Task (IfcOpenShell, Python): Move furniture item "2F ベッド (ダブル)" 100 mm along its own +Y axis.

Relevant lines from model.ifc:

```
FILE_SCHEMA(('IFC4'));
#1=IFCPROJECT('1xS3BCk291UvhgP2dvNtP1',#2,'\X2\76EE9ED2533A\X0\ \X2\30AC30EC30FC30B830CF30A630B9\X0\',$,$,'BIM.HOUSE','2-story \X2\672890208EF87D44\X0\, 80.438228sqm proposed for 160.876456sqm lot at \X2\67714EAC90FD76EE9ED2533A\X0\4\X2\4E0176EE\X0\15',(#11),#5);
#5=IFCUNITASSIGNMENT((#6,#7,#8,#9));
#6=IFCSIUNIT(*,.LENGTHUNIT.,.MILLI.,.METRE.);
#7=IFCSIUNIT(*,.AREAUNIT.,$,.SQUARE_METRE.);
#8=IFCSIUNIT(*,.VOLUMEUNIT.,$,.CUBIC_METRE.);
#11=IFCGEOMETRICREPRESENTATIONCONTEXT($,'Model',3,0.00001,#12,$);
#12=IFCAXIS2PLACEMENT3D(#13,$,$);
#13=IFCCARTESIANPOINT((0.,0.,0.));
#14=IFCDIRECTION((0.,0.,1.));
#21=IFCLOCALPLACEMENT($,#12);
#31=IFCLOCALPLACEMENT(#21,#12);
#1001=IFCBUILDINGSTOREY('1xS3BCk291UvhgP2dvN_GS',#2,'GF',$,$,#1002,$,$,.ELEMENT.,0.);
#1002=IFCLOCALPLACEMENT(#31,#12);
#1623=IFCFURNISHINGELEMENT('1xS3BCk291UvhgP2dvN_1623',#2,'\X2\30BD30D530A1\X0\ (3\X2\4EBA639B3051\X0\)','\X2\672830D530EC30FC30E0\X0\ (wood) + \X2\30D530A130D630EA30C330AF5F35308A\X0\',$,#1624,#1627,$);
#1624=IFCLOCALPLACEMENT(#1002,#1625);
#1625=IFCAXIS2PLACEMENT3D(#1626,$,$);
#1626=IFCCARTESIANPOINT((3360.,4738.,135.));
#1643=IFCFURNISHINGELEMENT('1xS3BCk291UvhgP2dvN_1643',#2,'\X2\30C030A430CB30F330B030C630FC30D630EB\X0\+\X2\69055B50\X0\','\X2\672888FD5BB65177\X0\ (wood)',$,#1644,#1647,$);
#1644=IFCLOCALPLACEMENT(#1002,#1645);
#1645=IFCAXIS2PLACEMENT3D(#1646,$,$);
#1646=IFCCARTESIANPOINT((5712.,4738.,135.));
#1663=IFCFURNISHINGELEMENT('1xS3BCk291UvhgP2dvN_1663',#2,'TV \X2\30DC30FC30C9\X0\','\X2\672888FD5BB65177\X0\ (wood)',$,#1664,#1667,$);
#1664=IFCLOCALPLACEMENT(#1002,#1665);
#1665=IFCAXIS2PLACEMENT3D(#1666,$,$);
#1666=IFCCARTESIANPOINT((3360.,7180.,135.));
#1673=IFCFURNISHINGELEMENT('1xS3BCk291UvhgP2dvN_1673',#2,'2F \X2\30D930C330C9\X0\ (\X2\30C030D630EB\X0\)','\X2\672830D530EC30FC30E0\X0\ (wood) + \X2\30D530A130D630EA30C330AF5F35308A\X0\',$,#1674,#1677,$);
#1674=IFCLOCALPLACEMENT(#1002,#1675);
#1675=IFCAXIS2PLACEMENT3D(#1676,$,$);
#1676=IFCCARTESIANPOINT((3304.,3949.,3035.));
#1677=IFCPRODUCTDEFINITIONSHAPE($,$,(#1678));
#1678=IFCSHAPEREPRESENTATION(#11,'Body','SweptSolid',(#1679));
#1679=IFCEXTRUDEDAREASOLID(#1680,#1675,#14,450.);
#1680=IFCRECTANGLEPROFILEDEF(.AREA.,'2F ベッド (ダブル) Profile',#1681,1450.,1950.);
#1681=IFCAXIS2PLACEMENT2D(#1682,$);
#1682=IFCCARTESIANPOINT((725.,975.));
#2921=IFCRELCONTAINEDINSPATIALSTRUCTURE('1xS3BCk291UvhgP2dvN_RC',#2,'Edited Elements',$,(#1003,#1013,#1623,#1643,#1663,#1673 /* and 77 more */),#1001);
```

```python
import ifcopenshell
import ifcopenshell.api.geometry
import ifcopenshell.util.placement
import ifcopenshell.util.unit

model = ifcopenshell.open("model.ifc")
unit_scale = ifcopenshell.util.unit.calculate_unit_scale(model)

item = model.by_guid("1xS3BCk291UvhgP2dvN_1673")
matrix = ifcopenshell.util.placement.get_local_placement(item.ObjectPlacement)
matrix[:3, 3] += matrix[:3, 1] * 0.1 / unit_scale
ifcopenshell.api.geometry.edit_object_placement(model, product=item, matrix=matrix, is_si=False)

print(ifcopenshell.util.placement.get_local_placement(item.ObjectPlacement).round(3) + 0.0)

model.write("model_edited.ifc")
```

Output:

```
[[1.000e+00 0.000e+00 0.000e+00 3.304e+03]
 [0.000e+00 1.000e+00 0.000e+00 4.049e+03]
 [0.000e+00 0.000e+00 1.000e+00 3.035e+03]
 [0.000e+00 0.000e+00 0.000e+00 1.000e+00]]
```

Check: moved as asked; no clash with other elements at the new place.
